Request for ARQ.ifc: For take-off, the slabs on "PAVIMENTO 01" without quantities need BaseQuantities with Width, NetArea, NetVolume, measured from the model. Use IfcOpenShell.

First a look at what the model holds.

```python
import ifcopenshell
import ifcopenshell.util.element
import ifcopenshell.util.unit

model = ifcopenshell.open("ARQ.ifc")
print(model.schema)
for unit_type in ("LENGTHUNIT", "AREAUNIT", "VOLUMEUNIT"):
    print(unit_type, ifcopenshell.util.unit.calculate_unit_scale(model, unit_type))
storey = next(s for s in model.by_type("IfcBuildingStorey") if s.Name == "PAVIMENTO 01")
slabs = [e for e in ifcopenshell.util.element.get_decomposition(storey) if e.is_a("IfcSlab")]
for e in sorted(slabs, key=lambda e: e.id()):
    print(e.id(), e.is_a(), e.Name, list(ifcopenshell.util.element.get_psets(e, qtos_only=True)), sep=" | ")
```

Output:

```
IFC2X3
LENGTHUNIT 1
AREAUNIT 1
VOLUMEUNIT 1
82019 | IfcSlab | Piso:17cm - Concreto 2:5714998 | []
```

```python
import ifcopenshell
import ifcopenshell.api.pset
import ifcopenshell.geom
import ifcopenshell.util.element
import ifcopenshell.util.shape
import ifcopenshell.util.unit

model = ifcopenshell.open("ARQ.ifc")
unit_scale = ifcopenshell.util.unit.calculate_unit_scale(model)
area_scale = ifcopenshell.util.unit.calculate_unit_scale(model, "AREAUNIT")
volume_scale = ifcopenshell.util.unit.calculate_unit_scale(model, "VOLUMEUNIT")
settings = ifcopenshell.geom.settings()

storey = next(s for s in model.by_type("IfcBuildingStorey") if s.Name == "PAVIMENTO 01")
slabs = [e for e in ifcopenshell.util.element.get_decomposition(storey) if e.is_a("IfcSlab")]

for e in sorted(slabs, key=lambda e: e.id()):
    if ifcopenshell.util.element.get_psets(e, qtos_only=True, should_inherit=False):
        continue
    # Geometry comes back in metres, in the element's own axes.
    shape = ifcopenshell.geom.create_shape(settings, e)
    values = {
        "Width": ifcopenshell.util.shape.get_z(shape.geometry) / unit_scale,
        "NetArea": ifcopenshell.util.shape.get_footprint_area(shape.geometry) / area_scale,
        "NetVolume": ifcopenshell.util.shape.get_volume(shape.geometry) / volume_scale,
    }
    qto = ifcopenshell.api.pset.add_qto(model, product=e, name="BaseQuantities")
    ifcopenshell.api.pset.edit_qto(model, qto=qto, properties=values)
    print(e.id(), {k: round(v, 3) for k, v in values.items()})

model.write("ARQ_rev.ifc")
```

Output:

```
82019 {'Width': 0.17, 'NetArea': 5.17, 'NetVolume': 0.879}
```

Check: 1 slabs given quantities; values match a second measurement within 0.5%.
